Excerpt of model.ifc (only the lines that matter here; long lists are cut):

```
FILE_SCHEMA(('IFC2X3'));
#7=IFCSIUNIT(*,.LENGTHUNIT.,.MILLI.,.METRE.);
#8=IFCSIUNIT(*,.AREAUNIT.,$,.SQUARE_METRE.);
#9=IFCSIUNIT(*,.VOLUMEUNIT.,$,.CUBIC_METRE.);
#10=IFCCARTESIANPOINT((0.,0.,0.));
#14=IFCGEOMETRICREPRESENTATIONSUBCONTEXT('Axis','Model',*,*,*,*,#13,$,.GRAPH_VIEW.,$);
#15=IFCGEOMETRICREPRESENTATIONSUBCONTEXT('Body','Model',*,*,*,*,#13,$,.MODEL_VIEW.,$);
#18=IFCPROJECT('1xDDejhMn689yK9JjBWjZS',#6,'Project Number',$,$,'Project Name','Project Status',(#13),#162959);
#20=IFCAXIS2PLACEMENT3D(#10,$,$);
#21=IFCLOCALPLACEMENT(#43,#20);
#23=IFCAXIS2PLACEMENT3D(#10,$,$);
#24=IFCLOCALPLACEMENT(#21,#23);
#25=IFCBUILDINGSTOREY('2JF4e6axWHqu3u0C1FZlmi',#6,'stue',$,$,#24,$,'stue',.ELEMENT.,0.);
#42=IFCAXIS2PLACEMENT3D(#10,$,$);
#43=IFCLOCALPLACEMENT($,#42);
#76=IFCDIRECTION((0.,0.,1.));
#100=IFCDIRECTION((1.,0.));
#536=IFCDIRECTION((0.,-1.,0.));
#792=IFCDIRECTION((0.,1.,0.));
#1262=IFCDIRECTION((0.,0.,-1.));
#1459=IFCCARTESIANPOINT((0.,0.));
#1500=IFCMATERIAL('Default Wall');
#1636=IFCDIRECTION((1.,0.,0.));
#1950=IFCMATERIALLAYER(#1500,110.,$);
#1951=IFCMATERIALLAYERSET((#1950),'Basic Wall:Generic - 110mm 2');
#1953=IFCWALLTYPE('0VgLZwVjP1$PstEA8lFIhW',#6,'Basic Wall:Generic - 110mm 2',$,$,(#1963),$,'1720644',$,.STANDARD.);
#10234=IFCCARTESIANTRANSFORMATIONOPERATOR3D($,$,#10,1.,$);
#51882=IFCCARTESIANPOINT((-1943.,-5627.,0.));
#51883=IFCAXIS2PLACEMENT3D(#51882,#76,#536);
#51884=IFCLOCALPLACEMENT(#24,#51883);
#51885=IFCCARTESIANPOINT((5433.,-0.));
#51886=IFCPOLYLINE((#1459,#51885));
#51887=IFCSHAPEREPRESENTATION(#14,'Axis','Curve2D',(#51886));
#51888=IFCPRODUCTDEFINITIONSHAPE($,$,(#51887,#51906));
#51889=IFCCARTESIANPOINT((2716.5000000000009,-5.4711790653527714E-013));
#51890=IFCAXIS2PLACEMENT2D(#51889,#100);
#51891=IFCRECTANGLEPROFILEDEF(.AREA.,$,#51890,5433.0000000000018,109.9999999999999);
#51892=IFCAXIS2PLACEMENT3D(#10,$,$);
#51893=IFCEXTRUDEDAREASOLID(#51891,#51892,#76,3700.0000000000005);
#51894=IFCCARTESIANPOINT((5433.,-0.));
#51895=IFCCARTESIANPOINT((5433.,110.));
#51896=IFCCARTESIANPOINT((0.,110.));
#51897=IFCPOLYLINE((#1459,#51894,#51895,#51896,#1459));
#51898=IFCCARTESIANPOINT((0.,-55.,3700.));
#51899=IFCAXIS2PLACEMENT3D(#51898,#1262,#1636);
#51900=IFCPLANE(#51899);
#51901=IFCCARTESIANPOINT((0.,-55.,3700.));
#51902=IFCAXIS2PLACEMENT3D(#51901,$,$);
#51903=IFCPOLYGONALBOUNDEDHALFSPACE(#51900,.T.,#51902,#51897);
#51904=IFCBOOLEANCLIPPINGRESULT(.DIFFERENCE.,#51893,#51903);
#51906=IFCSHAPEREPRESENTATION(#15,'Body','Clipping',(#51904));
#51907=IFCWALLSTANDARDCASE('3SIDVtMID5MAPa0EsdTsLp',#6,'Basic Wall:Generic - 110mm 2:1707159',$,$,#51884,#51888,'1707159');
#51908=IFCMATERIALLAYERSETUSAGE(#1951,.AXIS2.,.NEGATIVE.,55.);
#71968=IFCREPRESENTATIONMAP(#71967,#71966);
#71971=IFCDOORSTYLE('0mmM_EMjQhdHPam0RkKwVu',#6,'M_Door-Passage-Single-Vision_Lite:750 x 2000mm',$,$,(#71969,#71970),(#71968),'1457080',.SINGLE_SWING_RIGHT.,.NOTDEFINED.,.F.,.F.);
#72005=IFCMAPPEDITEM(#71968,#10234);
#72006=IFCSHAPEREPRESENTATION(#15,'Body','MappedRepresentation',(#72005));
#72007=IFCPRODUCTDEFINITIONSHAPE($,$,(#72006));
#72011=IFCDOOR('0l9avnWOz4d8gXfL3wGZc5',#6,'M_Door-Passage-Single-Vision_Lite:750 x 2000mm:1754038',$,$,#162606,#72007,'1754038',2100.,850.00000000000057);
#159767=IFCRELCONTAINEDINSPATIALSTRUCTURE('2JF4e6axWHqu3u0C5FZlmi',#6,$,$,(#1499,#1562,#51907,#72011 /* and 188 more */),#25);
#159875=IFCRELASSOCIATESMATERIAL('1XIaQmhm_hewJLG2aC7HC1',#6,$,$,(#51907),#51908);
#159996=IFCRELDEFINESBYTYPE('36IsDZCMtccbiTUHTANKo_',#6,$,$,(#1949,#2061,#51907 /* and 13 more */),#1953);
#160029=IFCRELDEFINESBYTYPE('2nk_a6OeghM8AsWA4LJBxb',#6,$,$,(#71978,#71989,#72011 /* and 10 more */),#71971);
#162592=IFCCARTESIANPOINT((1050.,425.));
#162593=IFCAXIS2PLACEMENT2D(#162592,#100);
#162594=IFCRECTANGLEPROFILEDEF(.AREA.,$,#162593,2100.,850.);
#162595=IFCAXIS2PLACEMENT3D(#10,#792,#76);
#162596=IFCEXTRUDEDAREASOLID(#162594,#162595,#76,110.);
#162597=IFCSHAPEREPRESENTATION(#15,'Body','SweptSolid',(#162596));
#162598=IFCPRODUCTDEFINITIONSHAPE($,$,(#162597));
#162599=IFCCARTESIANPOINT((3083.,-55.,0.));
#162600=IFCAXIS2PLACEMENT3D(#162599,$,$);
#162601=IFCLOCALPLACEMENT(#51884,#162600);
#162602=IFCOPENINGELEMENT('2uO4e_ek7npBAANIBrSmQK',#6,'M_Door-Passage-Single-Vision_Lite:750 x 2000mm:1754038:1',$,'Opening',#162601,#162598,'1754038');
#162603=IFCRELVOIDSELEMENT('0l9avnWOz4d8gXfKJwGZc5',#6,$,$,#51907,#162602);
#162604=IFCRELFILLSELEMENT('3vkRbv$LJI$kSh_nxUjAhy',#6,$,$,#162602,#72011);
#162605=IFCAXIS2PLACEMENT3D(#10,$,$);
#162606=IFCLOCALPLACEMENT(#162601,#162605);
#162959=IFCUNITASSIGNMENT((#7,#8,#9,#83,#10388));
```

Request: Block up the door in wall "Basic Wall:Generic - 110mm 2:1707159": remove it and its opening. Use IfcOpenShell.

```python
import ifcopenshell
import ifcopenshell.api.feature
import ifcopenshell.api.root
import ifcopenshell.geom
import ifcopenshell.util.shape

model = ifcopenshell.open("model.ifc")
settings = ifcopenshell.geom.settings()


def volume(element):
    """Net volume in cubic metres, openings subtracted."""
    shape = ifcopenshell.geom.create_shape(settings, element)
    return ifcopenshell.util.shape.get_volume(shape.geometry)


door = model.by_guid("0l9avnWOz4d8gXfL3wGZc5")
opening = door.FillsVoids[0].RelatingOpeningElement
wall = opening.VoidsElements[0].RelatingBuildingElement
before = volume(wall)

ifcopenshell.api.root.remove_product(model, product=door)
ifcopenshell.api.feature.remove_feature(model, feature=opening)

after = volume(wall)

print(f"wall volume {before:.3f} -> {after:.3f} m3")

model.write("model_updated.ifc")
```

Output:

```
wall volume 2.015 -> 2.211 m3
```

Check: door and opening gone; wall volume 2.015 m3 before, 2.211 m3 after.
